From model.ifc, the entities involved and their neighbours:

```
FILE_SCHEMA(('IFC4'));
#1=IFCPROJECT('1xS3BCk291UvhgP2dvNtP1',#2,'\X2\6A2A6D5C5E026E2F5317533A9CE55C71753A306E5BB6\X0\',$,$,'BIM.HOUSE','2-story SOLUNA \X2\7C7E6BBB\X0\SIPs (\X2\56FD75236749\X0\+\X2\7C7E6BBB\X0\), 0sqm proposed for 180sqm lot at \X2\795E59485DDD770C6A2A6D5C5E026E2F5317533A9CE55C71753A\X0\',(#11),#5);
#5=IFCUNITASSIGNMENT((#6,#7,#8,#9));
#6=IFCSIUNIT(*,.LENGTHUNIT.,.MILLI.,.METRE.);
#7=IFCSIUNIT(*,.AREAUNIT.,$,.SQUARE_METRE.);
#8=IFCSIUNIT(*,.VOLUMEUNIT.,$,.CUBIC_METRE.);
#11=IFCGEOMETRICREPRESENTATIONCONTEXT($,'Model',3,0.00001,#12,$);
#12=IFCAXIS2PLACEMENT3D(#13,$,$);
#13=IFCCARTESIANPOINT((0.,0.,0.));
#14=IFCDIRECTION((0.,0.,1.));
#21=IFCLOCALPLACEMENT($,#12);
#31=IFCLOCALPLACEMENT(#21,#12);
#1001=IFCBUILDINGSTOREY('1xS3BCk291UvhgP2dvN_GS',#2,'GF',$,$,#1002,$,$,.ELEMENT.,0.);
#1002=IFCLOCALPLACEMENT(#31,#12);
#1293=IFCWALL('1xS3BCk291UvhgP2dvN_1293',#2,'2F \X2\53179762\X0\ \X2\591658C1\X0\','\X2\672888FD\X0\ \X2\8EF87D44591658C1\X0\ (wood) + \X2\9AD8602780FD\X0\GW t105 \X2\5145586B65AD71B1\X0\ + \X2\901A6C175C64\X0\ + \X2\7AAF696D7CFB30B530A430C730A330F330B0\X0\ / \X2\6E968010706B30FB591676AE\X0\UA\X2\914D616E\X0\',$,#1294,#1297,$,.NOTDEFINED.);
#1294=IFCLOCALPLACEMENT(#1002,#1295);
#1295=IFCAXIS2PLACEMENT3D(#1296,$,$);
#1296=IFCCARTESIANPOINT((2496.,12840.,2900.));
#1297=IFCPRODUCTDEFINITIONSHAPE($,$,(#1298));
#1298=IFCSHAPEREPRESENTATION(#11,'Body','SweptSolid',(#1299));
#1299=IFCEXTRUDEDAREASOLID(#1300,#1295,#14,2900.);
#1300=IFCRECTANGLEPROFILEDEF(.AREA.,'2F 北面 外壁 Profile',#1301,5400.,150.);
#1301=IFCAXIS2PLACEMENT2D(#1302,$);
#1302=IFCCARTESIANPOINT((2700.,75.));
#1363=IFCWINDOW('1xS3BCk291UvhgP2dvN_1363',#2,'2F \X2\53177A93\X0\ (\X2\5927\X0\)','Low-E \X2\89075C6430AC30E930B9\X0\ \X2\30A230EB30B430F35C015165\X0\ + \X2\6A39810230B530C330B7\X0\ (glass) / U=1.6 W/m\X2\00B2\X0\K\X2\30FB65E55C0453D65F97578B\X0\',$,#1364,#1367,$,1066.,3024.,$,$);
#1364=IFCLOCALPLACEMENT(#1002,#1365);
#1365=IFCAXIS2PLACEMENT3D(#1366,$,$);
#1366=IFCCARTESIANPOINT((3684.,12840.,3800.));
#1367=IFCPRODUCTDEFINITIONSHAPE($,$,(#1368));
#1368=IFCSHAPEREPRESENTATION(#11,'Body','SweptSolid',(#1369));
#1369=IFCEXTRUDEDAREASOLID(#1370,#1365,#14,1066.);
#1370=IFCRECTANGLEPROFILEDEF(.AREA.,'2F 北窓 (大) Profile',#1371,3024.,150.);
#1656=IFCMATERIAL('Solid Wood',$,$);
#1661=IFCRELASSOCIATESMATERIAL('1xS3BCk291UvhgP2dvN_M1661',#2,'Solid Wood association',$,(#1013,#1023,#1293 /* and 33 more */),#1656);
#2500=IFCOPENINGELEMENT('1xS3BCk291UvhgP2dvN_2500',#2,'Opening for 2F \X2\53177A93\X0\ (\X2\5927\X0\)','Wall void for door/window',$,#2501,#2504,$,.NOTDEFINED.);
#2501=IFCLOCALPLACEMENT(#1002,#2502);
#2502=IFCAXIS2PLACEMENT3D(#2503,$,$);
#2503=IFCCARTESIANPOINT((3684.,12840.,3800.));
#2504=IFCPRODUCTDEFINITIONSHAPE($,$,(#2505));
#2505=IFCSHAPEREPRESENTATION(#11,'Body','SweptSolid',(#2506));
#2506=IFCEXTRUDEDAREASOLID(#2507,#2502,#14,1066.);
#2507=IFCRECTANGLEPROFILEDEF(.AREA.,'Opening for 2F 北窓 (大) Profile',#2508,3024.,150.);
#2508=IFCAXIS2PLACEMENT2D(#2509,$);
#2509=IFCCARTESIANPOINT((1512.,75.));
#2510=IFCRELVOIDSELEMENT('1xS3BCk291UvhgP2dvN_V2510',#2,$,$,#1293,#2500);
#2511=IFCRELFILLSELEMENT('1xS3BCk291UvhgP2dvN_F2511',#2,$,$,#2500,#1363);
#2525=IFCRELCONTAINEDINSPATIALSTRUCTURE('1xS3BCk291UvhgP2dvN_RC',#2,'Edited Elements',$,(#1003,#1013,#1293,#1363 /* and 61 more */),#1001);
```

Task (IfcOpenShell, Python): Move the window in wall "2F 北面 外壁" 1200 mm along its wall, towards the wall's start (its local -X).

```python
import ifcopenshell
import ifcopenshell.api.geometry
import ifcopenshell.util.placement

model = ifcopenshell.open("model.ifc")

window = model.by_guid("1xS3BCk291UvhgP2dvN_1363")
opening = window.FillsVoids[0].RelatingOpeningElement
wall = opening.VoidsElements[0].RelatingBuildingElement

wall_matrix = ifcopenshell.util.placement.get_local_placement(wall.ObjectPlacement)
shift = wall_matrix[:3, 0] * -1200.0
before = ifcopenshell.util.placement.get_local_placement(window.ObjectPlacement)[:3, 3].copy()

# The window is not placed relative to its opening, so move both.
for product in (opening, window):
    matrix = ifcopenshell.util.placement.get_local_placement(product.ObjectPlacement)
    matrix[:3, 3] += shift
    ifcopenshell.api.geometry.edit_object_placement(model, product=product, matrix=matrix, is_si=False)

after = ifcopenshell.util.placement.get_local_placement(window.ObjectPlacement)[:3, 3]
print("window moved by", (after - before).round(3) + 0.0)

model.write("model_rev.ifc")
```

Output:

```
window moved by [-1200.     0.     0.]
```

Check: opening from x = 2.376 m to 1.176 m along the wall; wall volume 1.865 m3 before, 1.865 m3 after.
